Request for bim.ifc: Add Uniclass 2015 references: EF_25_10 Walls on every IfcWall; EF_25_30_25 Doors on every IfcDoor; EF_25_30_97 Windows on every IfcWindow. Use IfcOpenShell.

First a look at what the model holds.

```python
import ifcopenshell

model = ifcopenshell.open("bim.ifc")
print(model.schema)
print("classifications:", [c.Name for c in model.by_type("IfcClassification")])
for ifc_class in ("IfcDoor", "IfcRoof", "IfcStair", "IfcWall", "IfcWindow"):
    print(ifc_class, len(model.by_type(ifc_class)))
```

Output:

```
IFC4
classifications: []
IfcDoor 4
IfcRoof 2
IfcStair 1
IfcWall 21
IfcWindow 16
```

```python
import ifcopenshell
import ifcopenshell.api.classification

model = ifcopenshell.open("bim.ifc")

system = ifcopenshell.api.classification.add_classification(model, classification="Uniclass 2015")

codes = {
    "IfcWall": ("EF_25_10", "Walls"),
    "IfcDoor": ("EF_25_30_25", "Doors"),
    "IfcWindow": ("EF_25_30_97", "Windows"),
}
for ifc_class, (code, name) in codes.items():
    products = model.by_type(ifc_class)
    ifcopenshell.api.classification.add_reference(
        model, products=products, classification=system, identification=code, name=name
    )
    print(code, len(products))

model.write("bim_edited.ifc")
```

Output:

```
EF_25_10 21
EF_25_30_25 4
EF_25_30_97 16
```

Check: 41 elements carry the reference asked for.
